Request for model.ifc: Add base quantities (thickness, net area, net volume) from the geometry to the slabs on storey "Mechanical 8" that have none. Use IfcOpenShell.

First a look at what the model holds.

```python
import ifcopenshell
import ifcopenshell.util.element
import ifcopenshell.util.unit

model = ifcopenshell.open("model.ifc")
print(model.schema)
for unit_type in ("LENGTHUNIT", "AREAUNIT", "VOLUMEUNIT"):
    print(unit_type, ifcopenshell.util.unit.calculate_unit_scale(model, unit_type))
storey = next(s for s in model.by_type("IfcBuildingStorey") if s.Name == "Mechanical 8")
slabs = [e for e in ifcopenshell.util.element.get_decomposition(storey) if e.is_a("IfcSlab")]
for e in sorted(slabs, key=lambda e: e.id()):
    print(e.id(), e.is_a(), e.Name, list(ifcopenshell.util.element.get_psets(e, qtos_only=True)), sep=" | ")
```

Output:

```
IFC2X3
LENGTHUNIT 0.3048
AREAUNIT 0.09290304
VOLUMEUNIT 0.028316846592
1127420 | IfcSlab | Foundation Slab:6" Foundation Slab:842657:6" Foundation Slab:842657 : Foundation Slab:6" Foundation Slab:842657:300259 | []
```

```python
import ifcopenshell
import ifcopenshell.api.pset
import ifcopenshell.geom
import ifcopenshell.util.element
import ifcopenshell.util.shape
import ifcopenshell.util.unit

model = ifcopenshell.open("model.ifc")
unit_scale = ifcopenshell.util.unit.calculate_unit_scale(model)
area_scale = ifcopenshell.util.unit.calculate_unit_scale(model, "AREAUNIT")
volume_scale = ifcopenshell.util.unit.calculate_unit_scale(model, "VOLUMEUNIT")
settings = ifcopenshell.geom.settings()

storey = next(s for s in model.by_type("IfcBuildingStorey") if s.Name == "Mechanical 8")
slabs = [e for e in ifcopenshell.util.element.get_decomposition(storey) if e.is_a("IfcSlab")]

for e in sorted(slabs, key=lambda e: e.id()):
    if ifcopenshell.util.element.get_psets(e, qtos_only=True, should_inherit=False):
        continue
    # Geometry comes back in metres, in the element's own axes.
    shape = ifcopenshell.geom.create_shape(settings, e)
    values = {
        "Width": ifcopenshell.util.shape.get_z(shape.geometry) / unit_scale,
        "NetArea": ifcopenshell.util.shape.get_footprint_area(shape.geometry) / area_scale,
        "NetVolume": ifcopenshell.util.shape.get_volume(shape.geometry) / volume_scale,
    }
    qto = ifcopenshell.api.pset.add_qto(model, product=e, name="BaseQuantities")
    ifcopenshell.api.pset.edit_qto(model, qto=qto, properties=values)
    print(e.id(), {k: round(v, 3) for k, v in values.items()})

model.write("model_edited.ifc")
```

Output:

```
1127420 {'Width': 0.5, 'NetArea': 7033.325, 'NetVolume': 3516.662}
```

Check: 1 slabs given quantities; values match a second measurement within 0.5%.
